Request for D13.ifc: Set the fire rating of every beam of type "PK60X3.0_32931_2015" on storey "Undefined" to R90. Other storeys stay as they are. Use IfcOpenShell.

First a look at what the model holds.

```python
import ifcopenshell
import ifcopenshell.util.element

model = ifcopenshell.open("D13.ifc")
print(model.schema)
storey = next(s for s in model.by_type("IfcBuildingStorey") if s.Name == "Undefined")
beams = [e for e in ifcopenshell.util.element.get_decomposition(storey) if e.is_a("IfcBeam")]
seen = {}
for e in beams:
    element_type = ifcopenshell.util.element.get_type(e)
    key = (element_type.Name if element_type != e and element_type else None, ifcopenshell.util.element.get_pset(e, "Pset_BeamCommon", "FireRating"))
    seen[key] = seen.get(key, 0) + 1
for (name, value), count in sorted(seen.items(), key=str):
    print(count, "x", name, "|", value)
```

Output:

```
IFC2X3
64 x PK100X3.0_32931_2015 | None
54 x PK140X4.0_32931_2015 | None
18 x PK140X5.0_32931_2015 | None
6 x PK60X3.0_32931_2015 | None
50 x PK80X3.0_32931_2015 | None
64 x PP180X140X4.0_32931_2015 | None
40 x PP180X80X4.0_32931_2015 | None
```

```python
import ifcopenshell
import ifcopenshell.api.pset
import ifcopenshell.util.element

model = ifcopenshell.open("D13.ifc")

storey = next(s for s in model.by_type("IfcBuildingStorey") if s.Name == "Undefined")
beams = [e for e in ifcopenshell.util.element.get_decomposition(storey) if e.is_a("IfcBeam")]

count = 0
for e in beams:
    element_type = ifcopenshell.util.element.get_type(e)
    if element_type in (None, e) or element_type.Name != "PK60X3.0_32931_2015":
        continue
    found = ifcopenshell.util.element.get_pset(e, "Pset_BeamCommon", should_inherit=False)
    if found:
        pset = model.by_id(found["id"])
        if len(ifcopenshell.util.element.get_elements_by_pset(pset)) > 1:
            pset = ifcopenshell.api.pset.unshare_pset(model, products=[e], pset=pset)[0]
    else:
        pset = ifcopenshell.api.pset.add_pset(model, product=e, name="Pset_BeamCommon")
    ifcopenshell.api.pset.edit_pset(model, pset=pset, properties={"FireRating": "R90"})
    count += 1

print(count, "beams updated")

model.write("D13-out.ifc")
```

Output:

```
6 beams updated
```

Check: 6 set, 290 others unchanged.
